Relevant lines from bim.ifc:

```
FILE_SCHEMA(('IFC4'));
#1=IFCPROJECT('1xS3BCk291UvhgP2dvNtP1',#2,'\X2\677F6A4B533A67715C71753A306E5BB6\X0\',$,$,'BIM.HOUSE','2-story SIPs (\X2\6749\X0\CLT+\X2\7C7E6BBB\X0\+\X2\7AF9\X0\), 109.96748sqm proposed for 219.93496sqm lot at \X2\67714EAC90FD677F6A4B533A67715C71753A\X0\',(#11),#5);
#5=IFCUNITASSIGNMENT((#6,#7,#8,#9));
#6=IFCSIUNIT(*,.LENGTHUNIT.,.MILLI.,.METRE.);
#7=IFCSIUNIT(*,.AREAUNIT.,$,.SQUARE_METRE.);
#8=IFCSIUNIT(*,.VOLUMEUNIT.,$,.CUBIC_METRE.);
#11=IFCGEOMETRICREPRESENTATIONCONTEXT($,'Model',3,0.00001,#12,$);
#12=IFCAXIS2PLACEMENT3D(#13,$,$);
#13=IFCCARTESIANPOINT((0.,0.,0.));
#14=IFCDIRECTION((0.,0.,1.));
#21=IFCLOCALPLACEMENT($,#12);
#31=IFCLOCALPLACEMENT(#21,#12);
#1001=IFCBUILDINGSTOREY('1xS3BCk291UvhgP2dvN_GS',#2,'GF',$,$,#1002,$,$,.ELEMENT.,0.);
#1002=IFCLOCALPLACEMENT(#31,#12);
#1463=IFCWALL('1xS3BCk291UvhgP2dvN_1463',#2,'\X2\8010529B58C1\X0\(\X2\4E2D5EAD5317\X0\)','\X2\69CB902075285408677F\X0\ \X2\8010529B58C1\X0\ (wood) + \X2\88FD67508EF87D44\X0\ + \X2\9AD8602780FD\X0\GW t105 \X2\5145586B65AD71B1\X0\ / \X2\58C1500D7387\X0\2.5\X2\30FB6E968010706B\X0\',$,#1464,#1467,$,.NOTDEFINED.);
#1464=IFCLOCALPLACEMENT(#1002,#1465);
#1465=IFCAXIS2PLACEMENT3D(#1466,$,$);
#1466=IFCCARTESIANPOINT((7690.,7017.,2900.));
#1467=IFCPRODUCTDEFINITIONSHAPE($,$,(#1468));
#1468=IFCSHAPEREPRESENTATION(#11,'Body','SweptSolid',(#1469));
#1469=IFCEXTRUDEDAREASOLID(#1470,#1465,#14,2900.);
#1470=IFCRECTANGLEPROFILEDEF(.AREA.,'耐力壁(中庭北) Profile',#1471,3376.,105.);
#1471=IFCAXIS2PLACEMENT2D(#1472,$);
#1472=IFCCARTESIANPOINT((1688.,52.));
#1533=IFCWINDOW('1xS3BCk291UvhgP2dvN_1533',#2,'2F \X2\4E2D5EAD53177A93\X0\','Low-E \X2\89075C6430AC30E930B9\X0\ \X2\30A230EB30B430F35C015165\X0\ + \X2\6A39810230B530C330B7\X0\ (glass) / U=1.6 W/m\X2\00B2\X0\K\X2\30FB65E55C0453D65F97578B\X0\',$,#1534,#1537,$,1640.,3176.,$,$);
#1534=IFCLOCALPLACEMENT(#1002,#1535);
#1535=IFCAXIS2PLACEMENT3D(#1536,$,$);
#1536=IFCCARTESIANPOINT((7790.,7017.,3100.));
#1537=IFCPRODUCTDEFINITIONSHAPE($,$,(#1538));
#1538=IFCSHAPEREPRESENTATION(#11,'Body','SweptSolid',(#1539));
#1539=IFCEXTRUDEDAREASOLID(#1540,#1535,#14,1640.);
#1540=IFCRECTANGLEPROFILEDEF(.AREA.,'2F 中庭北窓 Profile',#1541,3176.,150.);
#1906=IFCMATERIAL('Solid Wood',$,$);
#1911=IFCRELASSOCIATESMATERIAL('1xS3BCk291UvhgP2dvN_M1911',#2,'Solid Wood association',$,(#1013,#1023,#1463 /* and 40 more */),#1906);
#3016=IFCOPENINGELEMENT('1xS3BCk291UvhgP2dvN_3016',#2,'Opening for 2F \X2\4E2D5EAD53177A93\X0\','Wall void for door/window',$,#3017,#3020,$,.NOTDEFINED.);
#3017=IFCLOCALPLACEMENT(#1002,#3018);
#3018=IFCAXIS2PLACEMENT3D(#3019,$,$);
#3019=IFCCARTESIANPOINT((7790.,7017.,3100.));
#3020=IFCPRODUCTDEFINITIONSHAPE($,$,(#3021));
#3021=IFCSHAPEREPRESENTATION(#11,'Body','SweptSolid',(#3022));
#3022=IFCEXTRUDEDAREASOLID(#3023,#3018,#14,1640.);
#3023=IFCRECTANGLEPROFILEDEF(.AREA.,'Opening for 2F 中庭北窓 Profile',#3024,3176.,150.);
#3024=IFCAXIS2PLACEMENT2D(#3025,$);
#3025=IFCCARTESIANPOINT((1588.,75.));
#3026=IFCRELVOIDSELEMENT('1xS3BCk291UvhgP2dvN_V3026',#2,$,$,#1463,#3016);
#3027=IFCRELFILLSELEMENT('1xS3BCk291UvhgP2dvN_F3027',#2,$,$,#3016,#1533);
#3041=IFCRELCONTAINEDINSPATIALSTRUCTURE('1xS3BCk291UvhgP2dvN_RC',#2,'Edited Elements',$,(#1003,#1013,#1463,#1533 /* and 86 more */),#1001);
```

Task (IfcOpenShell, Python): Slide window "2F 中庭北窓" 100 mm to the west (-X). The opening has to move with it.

```python
import ifcopenshell
import ifcopenshell.api.geometry
import ifcopenshell.util.placement
import ifcopenshell.util.unit

model = ifcopenshell.open("bim.ifc")
unit_scale = ifcopenshell.util.unit.calculate_unit_scale(model)

window = model.by_guid("1xS3BCk291UvhgP2dvN_1533")
opening = window.FillsVoids[0].RelatingOpeningElement
wall = opening.VoidsElements[0].RelatingBuildingElement

wall_matrix = ifcopenshell.util.placement.get_local_placement(wall.ObjectPlacement)
shift = wall_matrix[:3, 0] * -0.1 / unit_scale
before = ifcopenshell.util.placement.get_local_placement(window.ObjectPlacement)[:3, 3].copy()

# The window is not placed relative to its opening, so move both.
for product in (opening, window):
    matrix = ifcopenshell.util.placement.get_local_placement(product.ObjectPlacement)
    matrix[:3, 3] += shift
    ifcopenshell.api.geometry.edit_object_placement(model, product=product, matrix=matrix, is_si=False)

after = ifcopenshell.util.placement.get_local_placement(window.ObjectPlacement)[:3, 3]
print("window moved by", (after - before).round(3) + 0.0)

model.write("bim_v2.ifc")
```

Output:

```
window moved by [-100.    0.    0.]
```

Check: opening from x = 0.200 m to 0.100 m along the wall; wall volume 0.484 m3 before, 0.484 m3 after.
